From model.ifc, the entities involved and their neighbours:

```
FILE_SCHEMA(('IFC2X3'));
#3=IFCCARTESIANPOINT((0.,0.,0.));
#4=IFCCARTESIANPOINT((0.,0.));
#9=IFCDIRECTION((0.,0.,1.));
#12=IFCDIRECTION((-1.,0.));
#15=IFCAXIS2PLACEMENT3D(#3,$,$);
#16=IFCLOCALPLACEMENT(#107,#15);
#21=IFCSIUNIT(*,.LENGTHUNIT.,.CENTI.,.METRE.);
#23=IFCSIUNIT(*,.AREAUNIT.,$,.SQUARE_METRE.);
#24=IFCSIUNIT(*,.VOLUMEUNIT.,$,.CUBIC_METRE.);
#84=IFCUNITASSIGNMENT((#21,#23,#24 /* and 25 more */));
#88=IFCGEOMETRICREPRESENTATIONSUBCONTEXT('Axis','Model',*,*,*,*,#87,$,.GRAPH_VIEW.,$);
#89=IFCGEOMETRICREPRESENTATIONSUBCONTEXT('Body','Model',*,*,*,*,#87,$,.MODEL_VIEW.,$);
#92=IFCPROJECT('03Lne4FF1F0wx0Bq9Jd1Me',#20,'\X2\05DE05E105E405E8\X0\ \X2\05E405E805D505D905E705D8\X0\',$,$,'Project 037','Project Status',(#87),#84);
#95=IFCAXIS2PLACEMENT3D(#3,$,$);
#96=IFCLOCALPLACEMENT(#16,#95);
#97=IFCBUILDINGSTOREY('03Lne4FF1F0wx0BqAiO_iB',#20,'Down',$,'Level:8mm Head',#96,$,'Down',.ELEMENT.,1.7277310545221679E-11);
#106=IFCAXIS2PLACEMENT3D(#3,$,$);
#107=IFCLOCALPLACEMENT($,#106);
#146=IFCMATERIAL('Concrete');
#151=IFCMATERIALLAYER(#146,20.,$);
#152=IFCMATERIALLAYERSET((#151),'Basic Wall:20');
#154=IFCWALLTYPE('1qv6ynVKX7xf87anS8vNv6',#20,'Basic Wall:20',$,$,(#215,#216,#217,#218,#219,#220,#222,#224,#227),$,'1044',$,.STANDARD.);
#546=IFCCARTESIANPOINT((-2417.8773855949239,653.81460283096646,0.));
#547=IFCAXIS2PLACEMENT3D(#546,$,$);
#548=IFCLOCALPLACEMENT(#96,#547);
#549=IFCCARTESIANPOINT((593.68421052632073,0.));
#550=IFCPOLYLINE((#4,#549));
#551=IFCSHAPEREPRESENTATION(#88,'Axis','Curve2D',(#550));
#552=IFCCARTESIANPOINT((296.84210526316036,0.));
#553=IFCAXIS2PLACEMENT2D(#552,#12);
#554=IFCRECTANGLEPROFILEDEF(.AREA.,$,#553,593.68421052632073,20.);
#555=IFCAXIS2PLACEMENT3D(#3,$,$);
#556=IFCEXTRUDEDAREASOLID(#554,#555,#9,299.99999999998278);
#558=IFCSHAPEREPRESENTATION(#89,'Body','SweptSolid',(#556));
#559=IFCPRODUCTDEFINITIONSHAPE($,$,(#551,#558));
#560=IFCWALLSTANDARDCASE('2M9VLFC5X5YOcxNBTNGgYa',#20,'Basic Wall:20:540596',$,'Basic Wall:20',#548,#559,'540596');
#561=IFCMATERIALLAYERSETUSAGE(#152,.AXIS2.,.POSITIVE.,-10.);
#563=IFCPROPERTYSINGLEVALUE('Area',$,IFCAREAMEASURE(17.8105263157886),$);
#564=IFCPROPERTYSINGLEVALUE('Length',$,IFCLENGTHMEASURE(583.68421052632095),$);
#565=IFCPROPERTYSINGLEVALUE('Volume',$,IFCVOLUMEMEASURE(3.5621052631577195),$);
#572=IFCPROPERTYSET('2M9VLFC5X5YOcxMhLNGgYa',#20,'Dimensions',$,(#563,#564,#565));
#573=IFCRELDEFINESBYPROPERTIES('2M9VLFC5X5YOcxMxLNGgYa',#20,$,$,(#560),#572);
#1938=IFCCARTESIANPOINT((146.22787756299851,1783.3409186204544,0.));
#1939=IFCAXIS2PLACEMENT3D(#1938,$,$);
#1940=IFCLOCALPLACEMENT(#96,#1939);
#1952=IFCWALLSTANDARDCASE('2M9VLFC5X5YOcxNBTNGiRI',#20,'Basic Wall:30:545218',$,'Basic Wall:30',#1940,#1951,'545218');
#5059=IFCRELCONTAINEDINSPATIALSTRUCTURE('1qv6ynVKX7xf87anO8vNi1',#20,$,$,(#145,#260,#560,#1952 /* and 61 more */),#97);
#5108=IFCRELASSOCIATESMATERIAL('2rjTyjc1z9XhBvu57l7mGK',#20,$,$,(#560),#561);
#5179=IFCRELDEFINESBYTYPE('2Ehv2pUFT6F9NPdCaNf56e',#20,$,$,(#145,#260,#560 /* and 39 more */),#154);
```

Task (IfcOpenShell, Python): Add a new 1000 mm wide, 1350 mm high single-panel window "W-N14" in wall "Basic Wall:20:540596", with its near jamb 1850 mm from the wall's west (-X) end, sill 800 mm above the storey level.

```python
import numpy as np
import ifcopenshell
import ifcopenshell.api.feature
import ifcopenshell.api.geometry
import ifcopenshell.api.pset
import ifcopenshell.api.root
import ifcopenshell.api.spatial
import ifcopenshell.api.type
import ifcopenshell.geom
import ifcopenshell.util.element
import ifcopenshell.util.placement
import ifcopenshell.util.representation
import ifcopenshell.util.shape
import ifcopenshell.util.unit

model = ifcopenshell.open("model.ifc")
unit_scale = ifcopenshell.util.unit.calculate_unit_scale(model)
area_scale = ifcopenshell.util.unit.calculate_unit_scale(model, "AREAUNIT")
volume_scale = ifcopenshell.util.unit.calculate_unit_scale(model, "VOLUMEUNIT")
settings = ifcopenshell.geom.settings()


def volume(element):
    """Net volume in cubic metres, openings subtracted."""
    shape = ifcopenshell.geom.create_shape(settings, element)
    return ifcopenshell.util.shape.get_volume(shape.geometry)


wall = model.by_guid("2M9VLFC5X5YOcxNBTNGgYa")
storey = ifcopenshell.util.element.get_container(wall, ifc_class="IfcBuildingStorey")
context = ifcopenshell.util.representation.get_context(model, "Model", "Body", "MODEL_VIEW")
before = volume(wall)

width, height, from_end, sill = 1, 1.35, 1.85, 0.8  # metres

# The wall runs along its own X axis, and the end named is its -X end.
wall_shape = ifcopenshell.geom.create_shape(settings, wall)
x, y, z = ifcopenshell.util.shape.get_vertices(wall_shape.geometry).T
start = x.min() + from_end
face, thickness = float(y.min()), float(y.max() - y.min())
wall_matrix = ifcopenshell.util.placement.get_local_placement(wall.ObjectPlacement)
level = ifcopenshell.util.placement.get_local_placement(storey.ObjectPlacement)[2, 3]


def in_wall(x, y):
    """Placement at x, y metres in the wall's axes, at sill height."""
    matrix = wall_matrix.copy()
    matrix[:, 3] = wall_matrix @ np.array([x / unit_scale, y / unit_scale, 0.0, 1.0])
    matrix[2, 3] = level + sill / unit_scale
    return matrix


# Opening: a box that overshoots both wall faces by 50 mm.
opening = ifcopenshell.api.root.create_entity(model, ifc_class="IfcOpeningElement")
box = ifcopenshell.api.geometry.add_wall_representation(
    model, context=context, length=width, height=height, thickness=thickness + 0.1
)
ifcopenshell.api.geometry.assign_representation(model, product=opening, representation=box)
ifcopenshell.api.geometry.edit_object_placement(model, product=opening, matrix=in_wall(start, face - 0.05), is_si=False)
ifcopenshell.api.feature.add_feature(model, feature=opening, element=wall)

window = ifcopenshell.api.root.create_entity(model, ifc_class="IfcWindow", name="W-N14")
window.OverallWidth, window.OverallHeight = width / unit_scale, height / unit_scale
body = ifcopenshell.api.geometry.add_window_representation(
    model,
    context=context,
    overall_width=window.OverallWidth,
    overall_height=window.OverallHeight,
    partition_type="SINGLE_PANEL",
)
ifcopenshell.api.geometry.assign_representation(model, product=window, representation=body)
ifcopenshell.api.spatial.assign_container(model, products=[window], relating_structure=storey)
fills = ifcopenshell.api.feature.add_filling(model, opening=opening, element=window)
fills.OwnerHistory = window.OwnerHistory  # required in IFC2X3

# IFC2X3 keeps the operation on the window style.
style = ifcopenshell.api.root.create_entity(model, ifc_class="IfcWindowStyle", name="W-N14")
style.OperationType, style.ConstructionType = "SINGLE_PANEL", "NOTDEFINED"
style.ParameterTakesPrecedence = style.Sizeable = False
ifcopenshell.api.type.assign_type(model, related_objects=[window], relating_type=style)

# Centre the window in the wall's thickness.
ifcopenshell.api.geometry.edit_object_placement(model, product=window, matrix=in_wall(start, face), is_si=False)
window_shape = ifcopenshell.geom.create_shape(settings, window)
depth = ifcopenshell.util.shape.get_vertices(window_shape.geometry)[:, 1]
offset = face + thickness / 2 - (depth.min() + depth.max()) / 2
ifcopenshell.api.geometry.edit_object_placement(model, product=window, matrix=in_wall(start, offset), is_si=False)

after = volume(wall)

# Update the wall's stored quantities.
pset = model.by_id(ifcopenshell.util.element.get_pset(wall, "Dimensions", should_inherit=False)["id"])
ifcopenshell.api.pset.edit_pset(model, pset=pset, properties={
    "Area": model.create_entity("IfcAreaMeasure", after / thickness / area_scale),
    "Volume": model.create_entity("IfcVolumeMeasure", after / volume_scale),
})

print(f"wall volume {before:.3f} -> {after:.3f} m3")

model.write("model_edited.ifc")
```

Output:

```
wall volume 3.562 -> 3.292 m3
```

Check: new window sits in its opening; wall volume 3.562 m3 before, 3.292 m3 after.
